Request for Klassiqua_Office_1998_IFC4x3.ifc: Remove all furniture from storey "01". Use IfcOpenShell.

First a look at what the model holds.

```python
import ifcopenshell
import ifcopenshell.util.element

model = ifcopenshell.open("Klassiqua_Office_1998_IFC4x3.ifc")
print(model.schema)
storey = next(s for s in model.by_type("IfcBuildingStorey") if s.Name == "01")
furniture = [e for e in ifcopenshell.util.element.get_decomposition(storey) if e.is_a("IfcFurnishingElement")]
seen = {}
for e in furniture:
    element_type = ifcopenshell.util.element.get_type(e)
    name = element_type.Name if element_type not in (None, e) else None
    seen[name] = seen.get(name, 0) + 1
for name, count in sorted(seen.items(), key=str):
    print(count, "x", name)
```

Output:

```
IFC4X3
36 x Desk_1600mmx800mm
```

```python
import ifcopenshell
import ifcopenshell.api.root
import ifcopenshell.util.element

model = ifcopenshell.open("Klassiqua_Office_1998_IFC4x3.ifc")

storey = next(s for s in model.by_type("IfcBuildingStorey") if s.Name == "01")
furniture = [e for e in ifcopenshell.util.element.get_decomposition(storey) if e.is_a("IfcFurnishingElement")]

for e in furniture:
    ifcopenshell.api.root.remove_product(model, product=e)
print(len(furniture), "removed")

model.write("Klassiqua_Office_1998_IFC4x3_rev.ifc")
```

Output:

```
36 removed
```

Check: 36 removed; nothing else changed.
